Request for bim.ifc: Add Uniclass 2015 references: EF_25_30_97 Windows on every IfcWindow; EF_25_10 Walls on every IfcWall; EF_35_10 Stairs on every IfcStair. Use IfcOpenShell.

First a look at what the model holds.

```python
import ifcopenshell

model = ifcopenshell.open("bim.ifc")
print(model.schema)
print("classifications:", [c.Name for c in model.by_type("IfcClassification")])
for ifc_class in ("IfcDoor", "IfcRoof", "IfcStair", "IfcWall", "IfcWindow"):
    print(ifc_class, len(model.by_type(ifc_class)))
```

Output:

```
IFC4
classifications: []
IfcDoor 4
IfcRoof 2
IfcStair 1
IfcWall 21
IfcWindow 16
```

```python
import ifcopenshell
import ifcopenshell.api.classification

model = ifcopenshell.open("bim.ifc")

system = ifcopenshell.api.classification.add_classification(model, classification="Uniclass 2015")

codes = {
    "IfcWindow": ("EF_25_30_97", "Windows"),
    "IfcWall": ("EF_25_10", "Walls"),
    "IfcStair": ("EF_35_10", "Stairs"),
}
for ifc_class, (code, name) in codes.items():
    products = model.by_type(ifc_class)
    ifcopenshell.api.classification.add_reference(
        model, products=products, classification=system, identification=code, name=name
    )
    print(code, len(products))

model.write("bim_updated.ifc")
```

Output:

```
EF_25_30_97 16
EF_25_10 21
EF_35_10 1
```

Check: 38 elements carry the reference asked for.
